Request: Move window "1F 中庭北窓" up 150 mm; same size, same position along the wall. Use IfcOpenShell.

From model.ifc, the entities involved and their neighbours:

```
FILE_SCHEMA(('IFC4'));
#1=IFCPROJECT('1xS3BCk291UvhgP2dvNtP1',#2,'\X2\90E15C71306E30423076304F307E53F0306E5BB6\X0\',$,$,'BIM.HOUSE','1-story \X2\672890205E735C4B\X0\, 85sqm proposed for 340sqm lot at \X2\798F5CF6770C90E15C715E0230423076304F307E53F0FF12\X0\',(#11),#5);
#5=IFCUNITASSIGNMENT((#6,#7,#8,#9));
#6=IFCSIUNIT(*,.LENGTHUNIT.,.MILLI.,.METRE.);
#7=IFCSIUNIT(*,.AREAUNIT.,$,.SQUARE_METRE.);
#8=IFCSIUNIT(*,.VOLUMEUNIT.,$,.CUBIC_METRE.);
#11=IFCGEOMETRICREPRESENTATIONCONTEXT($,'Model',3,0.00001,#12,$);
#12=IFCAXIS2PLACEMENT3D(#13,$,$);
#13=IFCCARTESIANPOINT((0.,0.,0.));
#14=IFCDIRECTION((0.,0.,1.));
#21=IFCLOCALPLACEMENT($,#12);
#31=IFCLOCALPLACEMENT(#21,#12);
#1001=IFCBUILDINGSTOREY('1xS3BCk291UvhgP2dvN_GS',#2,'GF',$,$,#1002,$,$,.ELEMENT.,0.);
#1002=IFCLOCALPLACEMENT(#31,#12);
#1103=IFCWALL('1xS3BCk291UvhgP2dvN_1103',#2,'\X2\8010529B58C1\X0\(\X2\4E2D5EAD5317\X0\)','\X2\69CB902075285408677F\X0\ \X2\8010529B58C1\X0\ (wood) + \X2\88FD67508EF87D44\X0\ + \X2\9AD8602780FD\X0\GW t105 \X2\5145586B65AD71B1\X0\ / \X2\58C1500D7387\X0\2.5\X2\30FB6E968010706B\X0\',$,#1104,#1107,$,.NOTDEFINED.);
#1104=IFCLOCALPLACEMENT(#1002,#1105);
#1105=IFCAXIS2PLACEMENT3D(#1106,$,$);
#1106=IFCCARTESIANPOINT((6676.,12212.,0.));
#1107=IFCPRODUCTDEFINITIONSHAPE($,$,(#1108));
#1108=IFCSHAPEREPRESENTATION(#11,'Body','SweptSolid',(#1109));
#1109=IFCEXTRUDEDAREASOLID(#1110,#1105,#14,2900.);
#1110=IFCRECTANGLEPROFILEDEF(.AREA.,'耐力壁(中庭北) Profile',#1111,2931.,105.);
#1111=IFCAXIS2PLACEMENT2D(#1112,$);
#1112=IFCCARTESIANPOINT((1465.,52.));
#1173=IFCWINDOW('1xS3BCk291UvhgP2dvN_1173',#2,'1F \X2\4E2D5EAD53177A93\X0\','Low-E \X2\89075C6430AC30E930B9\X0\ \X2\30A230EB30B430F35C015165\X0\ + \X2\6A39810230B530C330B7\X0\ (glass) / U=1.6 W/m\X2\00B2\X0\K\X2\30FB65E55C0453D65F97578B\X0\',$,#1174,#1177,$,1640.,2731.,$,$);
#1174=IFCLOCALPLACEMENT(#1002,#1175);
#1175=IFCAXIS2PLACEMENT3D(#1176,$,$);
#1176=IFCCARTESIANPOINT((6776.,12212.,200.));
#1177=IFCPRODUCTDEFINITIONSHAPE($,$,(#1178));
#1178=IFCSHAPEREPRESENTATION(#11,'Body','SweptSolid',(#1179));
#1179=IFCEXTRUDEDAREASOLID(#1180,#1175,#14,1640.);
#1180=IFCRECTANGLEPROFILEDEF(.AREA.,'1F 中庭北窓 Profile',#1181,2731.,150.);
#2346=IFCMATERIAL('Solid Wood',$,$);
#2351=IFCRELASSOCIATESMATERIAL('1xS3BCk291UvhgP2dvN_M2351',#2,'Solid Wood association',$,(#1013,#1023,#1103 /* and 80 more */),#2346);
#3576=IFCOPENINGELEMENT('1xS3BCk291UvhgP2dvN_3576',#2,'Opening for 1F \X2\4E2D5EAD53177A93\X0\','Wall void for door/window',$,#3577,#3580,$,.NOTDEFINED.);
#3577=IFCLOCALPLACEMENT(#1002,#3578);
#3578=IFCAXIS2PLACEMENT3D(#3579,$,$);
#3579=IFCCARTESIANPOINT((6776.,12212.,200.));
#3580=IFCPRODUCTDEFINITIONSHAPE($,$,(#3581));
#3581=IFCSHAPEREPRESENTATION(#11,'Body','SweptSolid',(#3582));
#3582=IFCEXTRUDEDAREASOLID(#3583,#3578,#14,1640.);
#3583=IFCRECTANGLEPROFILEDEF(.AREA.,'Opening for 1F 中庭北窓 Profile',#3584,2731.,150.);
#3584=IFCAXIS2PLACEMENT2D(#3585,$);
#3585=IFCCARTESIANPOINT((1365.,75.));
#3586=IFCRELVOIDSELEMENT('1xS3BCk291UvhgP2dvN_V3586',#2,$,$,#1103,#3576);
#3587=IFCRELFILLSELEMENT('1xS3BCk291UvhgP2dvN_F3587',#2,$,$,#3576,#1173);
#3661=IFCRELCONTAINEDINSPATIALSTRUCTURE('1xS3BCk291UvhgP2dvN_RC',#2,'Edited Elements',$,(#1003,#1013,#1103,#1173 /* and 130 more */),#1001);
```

```python
import numpy as np
import ifcopenshell
import ifcopenshell.api.geometry
import ifcopenshell.util.placement
import ifcopenshell.util.unit

model = ifcopenshell.open("model.ifc")
unit_scale = ifcopenshell.util.unit.calculate_unit_scale(model)

window = model.by_guid("1xS3BCk291UvhgP2dvN_1173")
opening = window.FillsVoids[0].RelatingOpeningElement
dz = 150.0

shift = np.array([0.0, 0.0, dz])
# The window is not placed relative to its opening, so move both.
for product in (opening, window):
    matrix = ifcopenshell.util.placement.get_local_placement(product.ObjectPlacement)
    matrix[:3, 3] += shift
    ifcopenshell.api.geometry.edit_object_placement(model, product=product, matrix=matrix, is_si=False)

print(f"moved by {dz * unit_scale:+.3f} m")

model.write("model_edited.ifc")
```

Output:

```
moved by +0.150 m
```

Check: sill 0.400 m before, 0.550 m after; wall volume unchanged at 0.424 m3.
